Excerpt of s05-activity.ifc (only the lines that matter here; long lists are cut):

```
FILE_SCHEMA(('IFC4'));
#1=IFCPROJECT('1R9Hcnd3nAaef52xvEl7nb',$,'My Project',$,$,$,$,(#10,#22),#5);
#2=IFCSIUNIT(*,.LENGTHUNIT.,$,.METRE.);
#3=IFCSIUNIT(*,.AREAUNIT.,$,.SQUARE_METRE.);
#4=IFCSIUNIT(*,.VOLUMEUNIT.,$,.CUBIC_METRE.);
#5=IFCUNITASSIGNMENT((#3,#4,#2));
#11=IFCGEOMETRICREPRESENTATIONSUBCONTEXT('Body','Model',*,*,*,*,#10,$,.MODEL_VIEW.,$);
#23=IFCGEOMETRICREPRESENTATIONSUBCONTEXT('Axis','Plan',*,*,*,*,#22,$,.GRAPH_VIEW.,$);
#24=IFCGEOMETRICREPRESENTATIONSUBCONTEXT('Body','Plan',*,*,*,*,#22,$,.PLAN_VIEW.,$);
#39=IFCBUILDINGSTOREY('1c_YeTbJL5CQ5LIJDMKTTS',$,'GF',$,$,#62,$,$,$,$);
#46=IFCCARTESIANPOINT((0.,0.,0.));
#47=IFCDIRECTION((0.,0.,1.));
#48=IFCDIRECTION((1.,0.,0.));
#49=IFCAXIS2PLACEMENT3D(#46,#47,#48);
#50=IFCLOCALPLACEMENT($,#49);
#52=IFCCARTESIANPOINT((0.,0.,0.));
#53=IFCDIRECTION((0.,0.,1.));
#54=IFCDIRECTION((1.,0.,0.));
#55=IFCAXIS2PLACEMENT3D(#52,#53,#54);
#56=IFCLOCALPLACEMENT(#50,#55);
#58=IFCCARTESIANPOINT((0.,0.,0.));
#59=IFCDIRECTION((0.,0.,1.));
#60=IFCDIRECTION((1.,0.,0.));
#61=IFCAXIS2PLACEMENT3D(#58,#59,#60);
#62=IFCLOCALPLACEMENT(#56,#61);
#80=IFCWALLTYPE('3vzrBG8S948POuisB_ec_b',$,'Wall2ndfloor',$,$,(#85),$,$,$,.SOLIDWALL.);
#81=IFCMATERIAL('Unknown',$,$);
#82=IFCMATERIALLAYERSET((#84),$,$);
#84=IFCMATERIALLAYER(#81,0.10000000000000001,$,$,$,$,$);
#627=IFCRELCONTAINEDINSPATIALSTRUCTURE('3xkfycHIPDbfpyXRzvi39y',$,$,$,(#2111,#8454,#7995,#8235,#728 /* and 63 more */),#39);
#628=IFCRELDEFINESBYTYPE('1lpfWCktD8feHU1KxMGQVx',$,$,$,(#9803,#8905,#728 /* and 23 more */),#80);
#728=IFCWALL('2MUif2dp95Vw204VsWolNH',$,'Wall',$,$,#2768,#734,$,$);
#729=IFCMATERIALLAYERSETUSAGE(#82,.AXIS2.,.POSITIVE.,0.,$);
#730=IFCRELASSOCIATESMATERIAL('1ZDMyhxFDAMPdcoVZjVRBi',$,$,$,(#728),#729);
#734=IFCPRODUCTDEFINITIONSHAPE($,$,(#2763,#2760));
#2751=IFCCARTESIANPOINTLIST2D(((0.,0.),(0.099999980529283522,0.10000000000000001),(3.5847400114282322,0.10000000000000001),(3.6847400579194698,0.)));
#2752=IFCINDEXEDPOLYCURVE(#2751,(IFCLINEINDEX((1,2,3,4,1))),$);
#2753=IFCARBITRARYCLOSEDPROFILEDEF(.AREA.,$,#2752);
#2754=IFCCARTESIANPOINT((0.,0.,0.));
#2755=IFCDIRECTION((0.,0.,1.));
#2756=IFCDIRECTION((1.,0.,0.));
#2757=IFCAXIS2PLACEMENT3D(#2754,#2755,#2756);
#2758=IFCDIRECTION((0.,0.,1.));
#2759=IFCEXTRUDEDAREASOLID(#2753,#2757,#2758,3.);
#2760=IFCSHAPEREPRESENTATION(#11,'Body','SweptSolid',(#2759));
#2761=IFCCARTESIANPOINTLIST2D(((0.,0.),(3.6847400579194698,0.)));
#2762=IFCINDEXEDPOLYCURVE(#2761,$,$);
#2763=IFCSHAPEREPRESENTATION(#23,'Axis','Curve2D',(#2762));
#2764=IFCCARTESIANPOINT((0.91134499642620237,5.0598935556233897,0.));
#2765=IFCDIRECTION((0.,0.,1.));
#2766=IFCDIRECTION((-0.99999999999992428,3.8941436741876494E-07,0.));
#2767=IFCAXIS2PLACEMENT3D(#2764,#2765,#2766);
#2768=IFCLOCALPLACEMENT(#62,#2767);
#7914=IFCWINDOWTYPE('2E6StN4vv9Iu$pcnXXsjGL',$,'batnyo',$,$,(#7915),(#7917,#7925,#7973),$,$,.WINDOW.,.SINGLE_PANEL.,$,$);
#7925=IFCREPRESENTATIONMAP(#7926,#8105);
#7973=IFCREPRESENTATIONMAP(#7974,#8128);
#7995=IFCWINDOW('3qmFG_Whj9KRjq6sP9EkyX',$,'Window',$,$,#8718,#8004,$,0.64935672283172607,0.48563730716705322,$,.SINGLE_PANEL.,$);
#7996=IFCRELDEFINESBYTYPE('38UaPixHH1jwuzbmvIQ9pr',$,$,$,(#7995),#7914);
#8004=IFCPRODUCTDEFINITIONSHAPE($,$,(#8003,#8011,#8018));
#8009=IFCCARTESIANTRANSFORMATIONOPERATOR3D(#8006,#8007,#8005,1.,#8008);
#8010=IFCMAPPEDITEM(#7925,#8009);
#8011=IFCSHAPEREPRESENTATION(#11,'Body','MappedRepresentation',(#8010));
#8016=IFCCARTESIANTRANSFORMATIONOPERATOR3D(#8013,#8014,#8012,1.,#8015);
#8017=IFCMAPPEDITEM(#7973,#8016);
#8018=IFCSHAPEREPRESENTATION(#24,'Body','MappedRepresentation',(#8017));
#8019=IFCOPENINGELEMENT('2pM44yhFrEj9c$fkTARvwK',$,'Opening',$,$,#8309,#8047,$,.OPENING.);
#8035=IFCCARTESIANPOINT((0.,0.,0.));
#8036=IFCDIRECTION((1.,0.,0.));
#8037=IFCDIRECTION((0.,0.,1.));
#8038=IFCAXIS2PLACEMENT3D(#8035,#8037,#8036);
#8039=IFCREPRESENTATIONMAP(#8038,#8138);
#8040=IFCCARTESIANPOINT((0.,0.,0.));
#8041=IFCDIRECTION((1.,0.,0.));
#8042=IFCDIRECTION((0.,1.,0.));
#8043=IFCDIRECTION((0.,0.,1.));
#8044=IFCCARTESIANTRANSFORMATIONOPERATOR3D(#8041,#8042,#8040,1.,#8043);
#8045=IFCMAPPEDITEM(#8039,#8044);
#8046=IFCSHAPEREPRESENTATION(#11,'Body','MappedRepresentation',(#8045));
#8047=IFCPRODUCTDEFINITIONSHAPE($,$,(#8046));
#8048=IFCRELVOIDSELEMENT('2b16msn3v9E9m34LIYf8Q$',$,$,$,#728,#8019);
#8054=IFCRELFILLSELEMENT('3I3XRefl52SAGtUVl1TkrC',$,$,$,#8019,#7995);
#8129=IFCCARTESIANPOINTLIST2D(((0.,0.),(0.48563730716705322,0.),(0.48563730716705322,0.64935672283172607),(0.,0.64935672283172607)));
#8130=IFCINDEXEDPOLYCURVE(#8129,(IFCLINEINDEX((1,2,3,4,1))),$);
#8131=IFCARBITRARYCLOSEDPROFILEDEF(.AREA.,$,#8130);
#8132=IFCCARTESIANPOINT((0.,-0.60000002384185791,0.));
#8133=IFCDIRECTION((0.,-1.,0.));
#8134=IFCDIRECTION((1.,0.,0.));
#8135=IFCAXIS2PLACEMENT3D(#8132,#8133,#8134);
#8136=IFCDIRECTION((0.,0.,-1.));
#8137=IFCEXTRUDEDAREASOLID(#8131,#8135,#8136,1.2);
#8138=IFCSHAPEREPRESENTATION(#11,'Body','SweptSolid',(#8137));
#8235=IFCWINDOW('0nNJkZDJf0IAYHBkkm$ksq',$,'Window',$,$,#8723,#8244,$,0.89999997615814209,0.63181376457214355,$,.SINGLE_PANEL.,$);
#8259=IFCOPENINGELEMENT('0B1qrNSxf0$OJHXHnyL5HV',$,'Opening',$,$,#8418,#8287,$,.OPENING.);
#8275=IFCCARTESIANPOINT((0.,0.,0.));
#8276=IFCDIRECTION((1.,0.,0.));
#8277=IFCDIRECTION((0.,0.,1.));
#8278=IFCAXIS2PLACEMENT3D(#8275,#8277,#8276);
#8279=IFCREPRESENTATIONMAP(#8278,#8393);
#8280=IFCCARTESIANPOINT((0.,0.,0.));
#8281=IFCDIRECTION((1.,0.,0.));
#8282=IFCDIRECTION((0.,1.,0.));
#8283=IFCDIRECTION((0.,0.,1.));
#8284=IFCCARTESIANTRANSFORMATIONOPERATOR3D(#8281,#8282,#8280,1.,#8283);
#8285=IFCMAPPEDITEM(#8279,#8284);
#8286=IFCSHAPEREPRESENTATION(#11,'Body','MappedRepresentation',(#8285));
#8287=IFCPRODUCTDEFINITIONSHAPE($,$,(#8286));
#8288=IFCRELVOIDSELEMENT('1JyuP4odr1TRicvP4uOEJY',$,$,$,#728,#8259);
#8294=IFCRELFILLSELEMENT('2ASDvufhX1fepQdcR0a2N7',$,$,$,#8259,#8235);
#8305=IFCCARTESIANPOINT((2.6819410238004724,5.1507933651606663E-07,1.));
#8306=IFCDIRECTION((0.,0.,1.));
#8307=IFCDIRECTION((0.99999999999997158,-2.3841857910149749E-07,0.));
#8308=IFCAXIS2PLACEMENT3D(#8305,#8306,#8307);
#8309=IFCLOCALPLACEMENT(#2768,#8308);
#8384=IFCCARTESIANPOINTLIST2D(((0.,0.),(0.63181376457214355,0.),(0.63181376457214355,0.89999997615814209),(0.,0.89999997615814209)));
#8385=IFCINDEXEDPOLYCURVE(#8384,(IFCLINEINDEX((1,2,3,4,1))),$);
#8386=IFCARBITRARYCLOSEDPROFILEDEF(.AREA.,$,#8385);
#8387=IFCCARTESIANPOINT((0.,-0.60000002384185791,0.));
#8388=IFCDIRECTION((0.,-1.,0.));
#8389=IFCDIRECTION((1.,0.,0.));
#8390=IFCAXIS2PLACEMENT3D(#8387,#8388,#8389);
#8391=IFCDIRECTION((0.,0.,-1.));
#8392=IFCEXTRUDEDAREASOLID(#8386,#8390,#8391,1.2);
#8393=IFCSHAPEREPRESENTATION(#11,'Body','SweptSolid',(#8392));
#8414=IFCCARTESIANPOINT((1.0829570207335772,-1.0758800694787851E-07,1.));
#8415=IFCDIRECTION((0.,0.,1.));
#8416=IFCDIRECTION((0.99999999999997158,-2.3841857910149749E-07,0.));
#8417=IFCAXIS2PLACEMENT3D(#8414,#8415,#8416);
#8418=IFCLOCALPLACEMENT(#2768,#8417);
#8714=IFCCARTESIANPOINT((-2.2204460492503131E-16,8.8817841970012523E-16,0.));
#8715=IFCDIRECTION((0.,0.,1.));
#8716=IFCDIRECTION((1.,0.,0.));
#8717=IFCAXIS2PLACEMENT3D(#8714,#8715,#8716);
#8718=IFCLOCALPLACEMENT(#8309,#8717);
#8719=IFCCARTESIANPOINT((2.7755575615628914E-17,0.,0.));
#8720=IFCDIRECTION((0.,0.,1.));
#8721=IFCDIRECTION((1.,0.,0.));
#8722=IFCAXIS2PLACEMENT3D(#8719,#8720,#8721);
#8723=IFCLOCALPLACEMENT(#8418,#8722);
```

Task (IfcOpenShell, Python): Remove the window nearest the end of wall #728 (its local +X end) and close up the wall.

```python
import ifcopenshell
import ifcopenshell.api.feature
import ifcopenshell.api.root
import ifcopenshell.geom
import ifcopenshell.util.shape

model = ifcopenshell.open("s05-activity.ifc")
settings = ifcopenshell.geom.settings()


def volume(element):
    """Net volume in cubic metres, openings subtracted."""
    shape = ifcopenshell.geom.create_shape(settings, element)
    return ifcopenshell.util.shape.get_volume(shape.geometry)


window = model.by_guid("3qmFG_Whj9KRjq6sP9EkyX")
opening = window.FillsVoids[0].RelatingOpeningElement
wall = opening.VoidsElements[0].RelatingBuildingElement
before = volume(wall)

ifcopenshell.api.root.remove_product(model, product=window)
ifcopenshell.api.feature.remove_feature(model, feature=opening)

after = volume(wall)

print(f"wall volume {before:.3f} -> {after:.3f} m3")

model.write("s05-activity_edited.ifc")
```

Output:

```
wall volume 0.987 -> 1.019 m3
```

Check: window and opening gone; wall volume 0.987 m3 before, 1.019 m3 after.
